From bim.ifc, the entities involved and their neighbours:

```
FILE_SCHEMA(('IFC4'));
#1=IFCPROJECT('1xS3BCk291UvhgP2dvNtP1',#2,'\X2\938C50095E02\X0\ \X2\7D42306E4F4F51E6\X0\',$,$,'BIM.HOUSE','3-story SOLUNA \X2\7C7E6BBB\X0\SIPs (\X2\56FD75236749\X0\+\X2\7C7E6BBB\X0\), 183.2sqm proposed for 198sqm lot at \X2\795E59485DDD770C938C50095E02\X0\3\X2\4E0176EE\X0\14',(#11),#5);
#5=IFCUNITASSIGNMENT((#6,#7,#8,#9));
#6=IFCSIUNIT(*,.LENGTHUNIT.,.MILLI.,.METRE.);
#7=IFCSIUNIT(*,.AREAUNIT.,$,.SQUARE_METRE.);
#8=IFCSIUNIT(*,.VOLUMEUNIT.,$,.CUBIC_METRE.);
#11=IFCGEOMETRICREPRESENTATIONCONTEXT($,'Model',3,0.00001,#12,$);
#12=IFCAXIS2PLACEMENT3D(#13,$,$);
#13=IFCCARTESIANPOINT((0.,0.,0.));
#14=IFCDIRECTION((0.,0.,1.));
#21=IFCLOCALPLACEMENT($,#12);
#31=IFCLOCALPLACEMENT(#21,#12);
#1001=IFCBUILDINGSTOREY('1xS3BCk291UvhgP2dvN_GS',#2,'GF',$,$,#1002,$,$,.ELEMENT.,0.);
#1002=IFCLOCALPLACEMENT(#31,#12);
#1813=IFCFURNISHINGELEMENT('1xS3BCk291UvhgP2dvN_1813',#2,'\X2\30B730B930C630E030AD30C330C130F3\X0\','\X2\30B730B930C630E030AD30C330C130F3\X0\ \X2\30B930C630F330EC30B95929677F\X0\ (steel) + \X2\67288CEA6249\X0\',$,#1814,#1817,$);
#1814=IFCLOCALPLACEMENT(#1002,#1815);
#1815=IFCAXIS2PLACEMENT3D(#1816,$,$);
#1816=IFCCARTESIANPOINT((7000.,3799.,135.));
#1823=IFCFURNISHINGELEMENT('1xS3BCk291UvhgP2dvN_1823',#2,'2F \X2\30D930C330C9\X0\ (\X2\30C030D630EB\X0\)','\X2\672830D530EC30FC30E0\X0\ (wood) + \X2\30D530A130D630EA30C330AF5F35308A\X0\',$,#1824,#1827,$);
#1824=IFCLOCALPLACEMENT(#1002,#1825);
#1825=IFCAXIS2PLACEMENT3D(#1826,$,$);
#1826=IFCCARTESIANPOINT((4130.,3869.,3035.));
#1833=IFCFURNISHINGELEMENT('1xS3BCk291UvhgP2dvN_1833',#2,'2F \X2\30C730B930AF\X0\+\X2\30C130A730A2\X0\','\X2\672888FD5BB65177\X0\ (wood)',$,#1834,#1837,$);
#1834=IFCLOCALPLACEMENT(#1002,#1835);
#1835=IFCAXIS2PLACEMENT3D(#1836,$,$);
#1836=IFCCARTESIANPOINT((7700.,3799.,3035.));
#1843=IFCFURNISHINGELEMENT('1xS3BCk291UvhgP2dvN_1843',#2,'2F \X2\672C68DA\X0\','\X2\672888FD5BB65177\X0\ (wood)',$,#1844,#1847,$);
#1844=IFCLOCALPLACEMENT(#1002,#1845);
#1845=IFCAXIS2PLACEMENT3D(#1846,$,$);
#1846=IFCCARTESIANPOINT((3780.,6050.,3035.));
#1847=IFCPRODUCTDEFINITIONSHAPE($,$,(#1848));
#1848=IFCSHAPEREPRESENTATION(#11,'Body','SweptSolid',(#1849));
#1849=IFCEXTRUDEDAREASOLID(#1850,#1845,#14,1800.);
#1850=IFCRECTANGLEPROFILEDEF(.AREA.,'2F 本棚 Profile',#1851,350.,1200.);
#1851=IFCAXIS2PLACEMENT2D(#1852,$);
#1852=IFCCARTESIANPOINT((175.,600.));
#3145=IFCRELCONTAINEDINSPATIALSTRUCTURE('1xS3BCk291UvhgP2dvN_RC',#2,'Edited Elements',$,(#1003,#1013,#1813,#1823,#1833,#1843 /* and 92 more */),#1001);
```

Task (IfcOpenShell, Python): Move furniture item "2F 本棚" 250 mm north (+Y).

```python
import ifcopenshell
import ifcopenshell.api.geometry
import ifcopenshell.util.placement

model = ifcopenshell.open("bim.ifc")

item = model.by_id(1843)
matrix = ifcopenshell.util.placement.get_local_placement(item.ObjectPlacement)
matrix[1, 3] += 250.0
ifcopenshell.api.geometry.edit_object_placement(model, product=item, matrix=matrix, is_si=False)

print(ifcopenshell.util.placement.get_local_placement(item.ObjectPlacement).round(3) + 0.0)

model.write("bim_updated.ifc")
```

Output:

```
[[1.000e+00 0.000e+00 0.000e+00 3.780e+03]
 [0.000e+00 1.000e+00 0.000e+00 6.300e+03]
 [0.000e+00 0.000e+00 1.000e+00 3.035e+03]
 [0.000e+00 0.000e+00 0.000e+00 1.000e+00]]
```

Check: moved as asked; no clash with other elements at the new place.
